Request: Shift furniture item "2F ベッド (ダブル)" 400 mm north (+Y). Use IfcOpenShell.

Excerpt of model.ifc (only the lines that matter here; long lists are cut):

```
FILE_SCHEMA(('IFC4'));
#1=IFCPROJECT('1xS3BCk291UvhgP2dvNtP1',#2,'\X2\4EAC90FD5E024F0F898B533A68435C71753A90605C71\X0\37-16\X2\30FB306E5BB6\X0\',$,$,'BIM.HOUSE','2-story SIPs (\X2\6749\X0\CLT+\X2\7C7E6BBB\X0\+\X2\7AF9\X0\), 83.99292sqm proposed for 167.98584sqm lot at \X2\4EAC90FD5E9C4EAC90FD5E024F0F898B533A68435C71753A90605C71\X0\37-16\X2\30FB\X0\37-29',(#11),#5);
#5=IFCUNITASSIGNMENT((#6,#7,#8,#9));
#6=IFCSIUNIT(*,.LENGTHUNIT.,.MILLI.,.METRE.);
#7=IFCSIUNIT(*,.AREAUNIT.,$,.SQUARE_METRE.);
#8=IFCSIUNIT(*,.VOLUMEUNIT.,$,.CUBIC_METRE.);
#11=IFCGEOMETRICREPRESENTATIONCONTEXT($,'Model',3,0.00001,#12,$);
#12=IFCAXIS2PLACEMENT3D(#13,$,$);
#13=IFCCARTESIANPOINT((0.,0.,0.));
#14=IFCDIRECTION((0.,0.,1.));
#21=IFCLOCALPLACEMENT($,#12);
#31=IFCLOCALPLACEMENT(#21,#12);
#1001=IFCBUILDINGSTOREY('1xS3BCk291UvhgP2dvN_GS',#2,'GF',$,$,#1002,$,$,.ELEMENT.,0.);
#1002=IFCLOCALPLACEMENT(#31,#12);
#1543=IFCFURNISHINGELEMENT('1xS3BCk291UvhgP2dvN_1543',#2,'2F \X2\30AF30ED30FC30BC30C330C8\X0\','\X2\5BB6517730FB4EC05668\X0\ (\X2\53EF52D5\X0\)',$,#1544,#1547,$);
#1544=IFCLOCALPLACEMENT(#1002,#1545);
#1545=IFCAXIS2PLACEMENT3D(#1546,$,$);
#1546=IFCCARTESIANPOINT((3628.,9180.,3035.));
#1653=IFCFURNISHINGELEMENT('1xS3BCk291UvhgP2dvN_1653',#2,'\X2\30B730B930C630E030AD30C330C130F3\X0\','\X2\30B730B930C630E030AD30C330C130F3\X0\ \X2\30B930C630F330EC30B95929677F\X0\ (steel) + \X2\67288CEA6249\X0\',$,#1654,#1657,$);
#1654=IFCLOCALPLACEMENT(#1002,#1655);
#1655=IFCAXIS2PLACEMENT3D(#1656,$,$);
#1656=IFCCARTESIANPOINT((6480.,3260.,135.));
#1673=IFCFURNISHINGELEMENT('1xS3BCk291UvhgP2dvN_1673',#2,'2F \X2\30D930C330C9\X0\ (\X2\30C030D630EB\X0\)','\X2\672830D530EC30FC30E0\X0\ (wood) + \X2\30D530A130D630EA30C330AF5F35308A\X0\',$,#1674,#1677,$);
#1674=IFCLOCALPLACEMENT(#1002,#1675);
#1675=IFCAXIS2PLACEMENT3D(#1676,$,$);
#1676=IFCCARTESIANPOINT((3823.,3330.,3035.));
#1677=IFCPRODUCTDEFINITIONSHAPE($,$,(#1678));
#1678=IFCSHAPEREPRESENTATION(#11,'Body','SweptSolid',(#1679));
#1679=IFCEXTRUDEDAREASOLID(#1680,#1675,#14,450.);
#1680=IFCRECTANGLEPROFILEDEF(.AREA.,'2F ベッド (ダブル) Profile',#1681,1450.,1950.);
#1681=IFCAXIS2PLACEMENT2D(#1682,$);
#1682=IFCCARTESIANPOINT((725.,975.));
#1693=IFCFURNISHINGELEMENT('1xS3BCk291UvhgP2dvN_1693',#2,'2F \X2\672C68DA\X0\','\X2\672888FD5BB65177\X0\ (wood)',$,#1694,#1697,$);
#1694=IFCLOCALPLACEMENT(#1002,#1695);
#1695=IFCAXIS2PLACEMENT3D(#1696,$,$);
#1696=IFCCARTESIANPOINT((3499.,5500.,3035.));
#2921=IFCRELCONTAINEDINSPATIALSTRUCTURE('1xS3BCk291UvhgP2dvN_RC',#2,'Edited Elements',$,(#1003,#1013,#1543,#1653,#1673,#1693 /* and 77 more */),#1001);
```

```python
import ifcopenshell
import ifcopenshell.api.geometry
import ifcopenshell.util.placement
import ifcopenshell.util.unit

model = ifcopenshell.open("model.ifc")
unit_scale = ifcopenshell.util.unit.calculate_unit_scale(model)

item = model.by_guid("1xS3BCk291UvhgP2dvN_1673")
matrix = ifcopenshell.util.placement.get_local_placement(item.ObjectPlacement)
matrix[1, 3] += 0.4 / unit_scale
ifcopenshell.api.geometry.edit_object_placement(model, product=item, matrix=matrix, is_si=False)

print(ifcopenshell.util.placement.get_local_placement(item.ObjectPlacement).round(3) + 0.0)

model.write("model-out.ifc")
```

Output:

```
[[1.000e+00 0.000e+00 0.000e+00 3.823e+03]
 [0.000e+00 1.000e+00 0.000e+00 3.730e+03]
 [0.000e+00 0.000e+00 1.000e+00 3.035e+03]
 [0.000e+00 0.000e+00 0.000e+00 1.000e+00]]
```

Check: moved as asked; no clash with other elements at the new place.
